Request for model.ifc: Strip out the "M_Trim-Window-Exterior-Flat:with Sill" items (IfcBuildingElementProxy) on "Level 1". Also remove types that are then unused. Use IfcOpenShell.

First a look at what the model holds.

```python
import ifcopenshell
import ifcopenshell.util.element

model = ifcopenshell.open("model.ifc")
print(model.schema)
storey = next(s for s in model.by_type("IfcBuildingStorey") if s.Name == "Level 1")
proxies = [e for e in ifcopenshell.util.element.get_decomposition(storey) if e.is_a("IfcBuildingElementProxy")]
seen = {}
for e in proxies:
    element_type = ifcopenshell.util.element.get_type(e)
    name = element_type.Name if element_type not in (None, e) else None
    seen[name] = seen.get(name, 0) + 1
for name, count in sorted(seen.items(), key=str):
    print(count, "x", name)
```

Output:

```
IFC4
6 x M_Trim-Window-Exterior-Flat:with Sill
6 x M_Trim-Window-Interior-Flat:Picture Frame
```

```python
import ifcopenshell
import ifcopenshell.api.root
import ifcopenshell.util.element

model = ifcopenshell.open("model.ifc")

storey = next(s for s in model.by_type("IfcBuildingStorey") if s.Name == "Level 1")
proxies = [e for e in ifcopenshell.util.element.get_decomposition(storey) if e.is_a("IfcBuildingElementProxy")]
targets = [e for e in proxies if (t := ifcopenshell.util.element.get_type(e)) not in (None, e) and t.Name == "M_Trim-Window-Exterior-Flat:with Sill"]
types = {ifcopenshell.util.element.get_type(e) for e in targets} - {None, *targets}

for e in targets:
    ifcopenshell.api.root.remove_product(model, product=e)
print(len(targets), "removed")

unused = [t for t in types if not ifcopenshell.util.element.get_types(t)]
for t in unused:
    ifcopenshell.api.root.remove_product(model, product=t)
print(len(unused), "unused types removed")

model.write("model_v2.ifc")
```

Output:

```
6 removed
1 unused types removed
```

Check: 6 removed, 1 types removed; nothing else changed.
